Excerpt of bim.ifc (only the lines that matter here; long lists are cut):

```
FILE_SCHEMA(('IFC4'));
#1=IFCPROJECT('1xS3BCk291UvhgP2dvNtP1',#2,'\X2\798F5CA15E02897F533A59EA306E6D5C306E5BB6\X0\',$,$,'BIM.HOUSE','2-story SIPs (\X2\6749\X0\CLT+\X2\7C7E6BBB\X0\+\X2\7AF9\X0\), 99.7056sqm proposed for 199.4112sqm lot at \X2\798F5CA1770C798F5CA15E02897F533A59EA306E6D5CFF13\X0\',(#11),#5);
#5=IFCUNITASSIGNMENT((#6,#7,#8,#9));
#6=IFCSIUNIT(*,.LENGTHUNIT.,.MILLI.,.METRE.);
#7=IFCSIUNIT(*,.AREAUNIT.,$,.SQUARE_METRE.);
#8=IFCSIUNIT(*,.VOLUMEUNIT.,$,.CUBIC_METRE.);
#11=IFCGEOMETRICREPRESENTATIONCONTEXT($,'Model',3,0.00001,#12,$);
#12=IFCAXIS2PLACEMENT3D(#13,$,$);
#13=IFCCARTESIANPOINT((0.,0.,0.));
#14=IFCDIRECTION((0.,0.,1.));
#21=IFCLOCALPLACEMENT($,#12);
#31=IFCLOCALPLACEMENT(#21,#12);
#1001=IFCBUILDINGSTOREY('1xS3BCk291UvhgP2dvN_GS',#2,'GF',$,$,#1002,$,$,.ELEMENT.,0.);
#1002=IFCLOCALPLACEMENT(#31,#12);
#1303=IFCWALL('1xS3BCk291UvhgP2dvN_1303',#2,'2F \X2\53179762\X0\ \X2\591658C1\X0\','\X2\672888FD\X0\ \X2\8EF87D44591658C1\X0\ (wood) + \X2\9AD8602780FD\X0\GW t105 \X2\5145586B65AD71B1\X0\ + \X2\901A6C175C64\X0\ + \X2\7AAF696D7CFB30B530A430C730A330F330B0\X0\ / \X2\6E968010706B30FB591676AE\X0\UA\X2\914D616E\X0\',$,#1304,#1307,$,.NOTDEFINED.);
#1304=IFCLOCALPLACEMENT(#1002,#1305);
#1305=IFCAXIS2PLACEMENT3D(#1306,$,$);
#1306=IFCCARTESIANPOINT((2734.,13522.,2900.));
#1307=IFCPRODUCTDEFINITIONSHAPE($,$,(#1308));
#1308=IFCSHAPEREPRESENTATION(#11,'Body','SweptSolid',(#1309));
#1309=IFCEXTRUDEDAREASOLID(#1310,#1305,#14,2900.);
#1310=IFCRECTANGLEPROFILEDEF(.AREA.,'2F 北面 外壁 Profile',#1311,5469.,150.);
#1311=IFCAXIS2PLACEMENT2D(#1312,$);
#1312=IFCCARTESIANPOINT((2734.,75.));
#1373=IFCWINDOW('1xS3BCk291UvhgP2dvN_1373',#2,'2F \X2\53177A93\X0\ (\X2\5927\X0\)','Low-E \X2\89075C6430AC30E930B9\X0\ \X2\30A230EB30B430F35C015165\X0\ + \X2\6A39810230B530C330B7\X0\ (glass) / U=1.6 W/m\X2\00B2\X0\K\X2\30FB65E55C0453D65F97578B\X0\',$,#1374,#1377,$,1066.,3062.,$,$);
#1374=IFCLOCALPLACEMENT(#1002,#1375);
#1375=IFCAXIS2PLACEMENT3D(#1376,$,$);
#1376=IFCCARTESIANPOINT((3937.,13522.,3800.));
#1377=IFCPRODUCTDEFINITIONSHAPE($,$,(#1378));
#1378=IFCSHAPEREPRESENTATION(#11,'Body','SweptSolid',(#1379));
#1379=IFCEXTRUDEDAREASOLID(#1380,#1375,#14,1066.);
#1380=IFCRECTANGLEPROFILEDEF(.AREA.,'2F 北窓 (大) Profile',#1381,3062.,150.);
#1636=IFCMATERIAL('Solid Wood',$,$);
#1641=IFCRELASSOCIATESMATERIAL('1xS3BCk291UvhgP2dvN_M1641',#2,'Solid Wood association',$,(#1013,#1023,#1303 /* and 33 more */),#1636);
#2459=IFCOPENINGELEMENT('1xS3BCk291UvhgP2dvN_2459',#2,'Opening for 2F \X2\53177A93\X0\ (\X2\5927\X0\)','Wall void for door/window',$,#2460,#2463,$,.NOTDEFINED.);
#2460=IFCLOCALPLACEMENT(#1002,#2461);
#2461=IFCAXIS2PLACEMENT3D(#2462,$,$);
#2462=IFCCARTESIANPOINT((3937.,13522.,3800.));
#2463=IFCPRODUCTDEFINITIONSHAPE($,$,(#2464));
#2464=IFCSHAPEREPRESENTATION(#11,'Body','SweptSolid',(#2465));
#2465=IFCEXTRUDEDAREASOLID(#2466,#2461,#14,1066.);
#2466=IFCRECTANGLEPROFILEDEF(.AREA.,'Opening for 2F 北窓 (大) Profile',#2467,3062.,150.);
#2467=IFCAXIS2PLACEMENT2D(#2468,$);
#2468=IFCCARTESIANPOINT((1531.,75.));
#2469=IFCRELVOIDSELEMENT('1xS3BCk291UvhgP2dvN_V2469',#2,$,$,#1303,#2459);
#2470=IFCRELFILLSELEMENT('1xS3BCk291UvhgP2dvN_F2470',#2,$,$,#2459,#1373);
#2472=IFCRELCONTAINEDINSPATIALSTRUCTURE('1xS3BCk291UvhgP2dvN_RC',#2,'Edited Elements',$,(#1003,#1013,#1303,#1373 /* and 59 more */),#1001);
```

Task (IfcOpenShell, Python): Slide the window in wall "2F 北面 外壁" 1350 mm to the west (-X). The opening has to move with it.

```python
import ifcopenshell
import ifcopenshell.api.geometry
import ifcopenshell.util.placement

model = ifcopenshell.open("bim.ifc")

window = model.by_guid("1xS3BCk291UvhgP2dvN_1373")
opening = window.FillsVoids[0].RelatingOpeningElement
wall = opening.VoidsElements[0].RelatingBuildingElement

wall_matrix = ifcopenshell.util.placement.get_local_placement(wall.ObjectPlacement)
shift = wall_matrix[:3, 0] * -1350.0
before = ifcopenshell.util.placement.get_local_placement(window.ObjectPlacement)[:3, 3].copy()

# The window is not placed relative to its opening, so move both.
for product in (opening, window):
    matrix = ifcopenshell.util.placement.get_local_placement(product.ObjectPlacement)
    matrix[:3, 3] += shift
    ifcopenshell.api.geometry.edit_object_placement(model, product=product, matrix=matrix, is_si=False)

after = ifcopenshell.util.placement.get_local_placement(window.ObjectPlacement)[:3, 3]
print("window moved by", (after - before).round(3) + 0.0)

model.write("bim_edited.ifc")
```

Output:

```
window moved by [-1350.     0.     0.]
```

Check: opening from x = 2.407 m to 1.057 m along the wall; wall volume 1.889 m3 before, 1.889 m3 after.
